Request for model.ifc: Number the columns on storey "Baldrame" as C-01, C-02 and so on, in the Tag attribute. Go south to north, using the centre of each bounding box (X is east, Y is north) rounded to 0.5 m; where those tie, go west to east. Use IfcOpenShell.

First a look at what the model holds.

```python
import ifcopenshell
import ifcopenshell.util.element
import ifcopenshell.util.placement

model = ifcopenshell.open("model.ifc")
print(model.schema)
storey = next(s for s in model.by_type("IfcBuildingStorey") if s.Name == "Baldrame")
columns = [e for e in ifcopenshell.util.element.get_decomposition(storey) if e.is_a("IfcColumn")]
for e in sorted(columns, key=lambda e: e.id()):
    origin = ifcopenshell.util.placement.get_local_placement(e.ObjectPlacement)[:3, 3]
    print(e.id(), e.Tag, e.Name, origin.round(2) + 0.0, sep=" | ")
```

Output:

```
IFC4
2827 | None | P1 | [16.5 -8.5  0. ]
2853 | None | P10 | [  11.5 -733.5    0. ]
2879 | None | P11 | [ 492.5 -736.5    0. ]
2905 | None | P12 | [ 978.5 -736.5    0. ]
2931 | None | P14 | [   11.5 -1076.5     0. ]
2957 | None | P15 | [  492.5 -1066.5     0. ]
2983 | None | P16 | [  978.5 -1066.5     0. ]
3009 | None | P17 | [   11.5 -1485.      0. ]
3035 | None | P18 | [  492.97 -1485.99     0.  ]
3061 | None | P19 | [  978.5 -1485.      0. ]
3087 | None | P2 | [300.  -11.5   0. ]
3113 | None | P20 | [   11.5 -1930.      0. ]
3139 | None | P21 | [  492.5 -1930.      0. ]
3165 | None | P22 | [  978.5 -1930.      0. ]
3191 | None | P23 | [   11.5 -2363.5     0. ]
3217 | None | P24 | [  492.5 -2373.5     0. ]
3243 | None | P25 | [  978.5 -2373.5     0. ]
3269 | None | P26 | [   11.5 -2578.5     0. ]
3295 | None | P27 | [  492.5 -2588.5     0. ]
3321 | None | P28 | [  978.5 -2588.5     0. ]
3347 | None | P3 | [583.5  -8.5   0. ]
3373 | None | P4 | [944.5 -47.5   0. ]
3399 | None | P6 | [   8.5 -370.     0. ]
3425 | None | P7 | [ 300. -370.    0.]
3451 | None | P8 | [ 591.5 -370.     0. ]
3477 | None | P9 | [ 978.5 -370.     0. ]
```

```python
import ifcopenshell
import ifcopenshell.geom
import ifcopenshell.util.element
import ifcopenshell.util.shape

model = ifcopenshell.open("model.ifc")
settings = ifcopenshell.geom.settings()
settings.set("use-world-coords", True)


def centre(element):
    shape = ifcopenshell.geom.create_shape(settings, element)
    return ifcopenshell.util.shape.get_bbox_centroid(shape.geometry)


storey = next(s for s in model.by_type("IfcBuildingStorey") if s.Name == "Baldrame")
columns = [e for e in ifcopenshell.util.element.get_decomposition(storey) if e.is_a("IfcColumn")]

# Insertion points can sit at a corner or the storey origin, so sort by the geometry (in metres).
centres = {e: centre(e) for e in columns}
columns.sort(key=lambda e: (round(centres[e][1] / 0.5), centres[e][0]))

for i, e in enumerate(columns, start=1):
    number = f"C-{i:02d}"
    e.Tag = number
    print(e.id(), number)

model.write("model_rev.ifc")
```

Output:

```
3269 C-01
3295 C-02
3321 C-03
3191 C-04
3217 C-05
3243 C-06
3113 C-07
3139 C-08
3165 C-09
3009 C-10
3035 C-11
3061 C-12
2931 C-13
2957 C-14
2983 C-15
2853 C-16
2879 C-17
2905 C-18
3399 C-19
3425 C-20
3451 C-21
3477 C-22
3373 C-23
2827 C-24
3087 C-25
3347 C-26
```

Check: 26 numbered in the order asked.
